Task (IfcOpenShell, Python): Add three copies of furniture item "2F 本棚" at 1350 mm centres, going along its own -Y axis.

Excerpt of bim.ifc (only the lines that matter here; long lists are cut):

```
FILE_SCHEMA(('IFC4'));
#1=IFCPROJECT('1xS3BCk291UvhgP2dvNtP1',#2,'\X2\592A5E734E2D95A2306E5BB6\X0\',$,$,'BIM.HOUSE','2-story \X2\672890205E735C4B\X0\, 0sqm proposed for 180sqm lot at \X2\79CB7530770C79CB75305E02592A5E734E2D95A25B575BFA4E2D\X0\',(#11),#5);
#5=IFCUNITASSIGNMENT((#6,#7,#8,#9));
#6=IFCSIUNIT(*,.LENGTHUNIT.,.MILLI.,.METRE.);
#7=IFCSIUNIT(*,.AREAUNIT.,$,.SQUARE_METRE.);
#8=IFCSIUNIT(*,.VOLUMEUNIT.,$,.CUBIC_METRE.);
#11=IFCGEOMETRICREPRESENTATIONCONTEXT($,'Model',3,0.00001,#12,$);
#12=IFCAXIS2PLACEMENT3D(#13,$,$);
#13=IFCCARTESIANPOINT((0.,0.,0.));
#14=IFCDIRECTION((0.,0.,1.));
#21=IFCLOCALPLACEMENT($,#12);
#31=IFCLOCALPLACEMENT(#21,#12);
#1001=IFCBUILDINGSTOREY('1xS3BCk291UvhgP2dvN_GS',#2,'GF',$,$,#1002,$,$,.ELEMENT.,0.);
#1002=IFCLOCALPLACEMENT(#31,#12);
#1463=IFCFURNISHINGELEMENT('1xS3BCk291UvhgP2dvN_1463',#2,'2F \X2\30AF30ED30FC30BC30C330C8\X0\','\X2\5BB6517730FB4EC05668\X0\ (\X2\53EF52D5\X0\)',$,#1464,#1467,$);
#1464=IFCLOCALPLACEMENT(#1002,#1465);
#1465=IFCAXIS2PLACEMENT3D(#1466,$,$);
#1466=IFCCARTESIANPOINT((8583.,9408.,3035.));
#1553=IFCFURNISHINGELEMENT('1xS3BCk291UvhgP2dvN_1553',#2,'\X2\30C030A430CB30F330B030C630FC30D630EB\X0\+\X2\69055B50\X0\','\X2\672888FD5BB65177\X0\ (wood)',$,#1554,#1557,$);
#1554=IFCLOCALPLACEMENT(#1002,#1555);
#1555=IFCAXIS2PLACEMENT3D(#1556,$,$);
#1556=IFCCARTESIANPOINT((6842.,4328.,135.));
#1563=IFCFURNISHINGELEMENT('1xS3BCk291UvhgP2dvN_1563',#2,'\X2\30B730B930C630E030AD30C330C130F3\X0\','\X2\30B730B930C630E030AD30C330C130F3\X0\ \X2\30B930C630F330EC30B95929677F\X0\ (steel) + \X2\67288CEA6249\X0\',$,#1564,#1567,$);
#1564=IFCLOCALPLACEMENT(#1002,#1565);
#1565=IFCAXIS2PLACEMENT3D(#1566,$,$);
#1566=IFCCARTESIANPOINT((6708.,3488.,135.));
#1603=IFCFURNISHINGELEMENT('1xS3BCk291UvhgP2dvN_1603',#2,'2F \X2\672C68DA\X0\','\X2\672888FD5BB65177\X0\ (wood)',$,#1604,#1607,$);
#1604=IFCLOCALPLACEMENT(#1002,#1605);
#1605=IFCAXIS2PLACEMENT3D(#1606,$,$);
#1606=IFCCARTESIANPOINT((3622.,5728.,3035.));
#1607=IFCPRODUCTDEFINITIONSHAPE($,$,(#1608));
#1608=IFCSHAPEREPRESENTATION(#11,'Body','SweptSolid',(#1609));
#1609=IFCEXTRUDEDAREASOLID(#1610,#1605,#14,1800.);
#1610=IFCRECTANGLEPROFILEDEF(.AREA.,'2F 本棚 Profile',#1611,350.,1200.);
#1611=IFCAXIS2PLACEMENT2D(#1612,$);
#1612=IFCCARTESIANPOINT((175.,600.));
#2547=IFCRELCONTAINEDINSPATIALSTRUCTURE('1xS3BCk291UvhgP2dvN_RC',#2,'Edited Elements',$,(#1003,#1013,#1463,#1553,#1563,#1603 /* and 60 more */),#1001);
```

```python
import ifcopenshell
import ifcopenshell.api.geometry
import ifcopenshell.api.root
import ifcopenshell.util.element
import ifcopenshell.util.placement
import ifcopenshell.util.unit

model = ifcopenshell.open("bim.ifc")
unit_scale = ifcopenshell.util.unit.calculate_unit_scale(model)


def reuse_history(source, copy):
    """copy_class also copies each property set's owner history, people and application; keep the originals."""
    for rel in copy.IsDefinedBy:
        if rel.is_a("IfcRelDefinesByProperties") and (history := rel.RelatingPropertyDefinition.OwnerHistory):
            rel.RelatingPropertyDefinition.OwnerHistory = source.OwnerHistory
            ifcopenshell.util.element.remove_deep2(model, history)


source = model.by_id(1603)
base = ifcopenshell.util.placement.get_local_placement(source.ObjectPlacement)
step = -base[:3, 1] * 1.35 / unit_scale

for i in range(1, 4):
    copy = ifcopenshell.api.root.copy_class(model, product=source)
    copy.Representation = ifcopenshell.util.element.copy_deep(
        model, source.Representation, exclude=["IfcGeometricRepresentationContext", "IfcRepresentationMap"]
    )
    reuse_history(source, copy)
    matrix = base.copy()
    matrix[:3, 3] += i * step
    print("added at", matrix[:3, 3].round(3) + 0.0)
    ifcopenshell.api.geometry.edit_object_placement(model, product=copy, matrix=matrix, is_si=False)

model.write("bim-out.ifc")
```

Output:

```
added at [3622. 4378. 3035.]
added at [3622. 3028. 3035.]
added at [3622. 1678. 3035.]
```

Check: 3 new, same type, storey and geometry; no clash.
